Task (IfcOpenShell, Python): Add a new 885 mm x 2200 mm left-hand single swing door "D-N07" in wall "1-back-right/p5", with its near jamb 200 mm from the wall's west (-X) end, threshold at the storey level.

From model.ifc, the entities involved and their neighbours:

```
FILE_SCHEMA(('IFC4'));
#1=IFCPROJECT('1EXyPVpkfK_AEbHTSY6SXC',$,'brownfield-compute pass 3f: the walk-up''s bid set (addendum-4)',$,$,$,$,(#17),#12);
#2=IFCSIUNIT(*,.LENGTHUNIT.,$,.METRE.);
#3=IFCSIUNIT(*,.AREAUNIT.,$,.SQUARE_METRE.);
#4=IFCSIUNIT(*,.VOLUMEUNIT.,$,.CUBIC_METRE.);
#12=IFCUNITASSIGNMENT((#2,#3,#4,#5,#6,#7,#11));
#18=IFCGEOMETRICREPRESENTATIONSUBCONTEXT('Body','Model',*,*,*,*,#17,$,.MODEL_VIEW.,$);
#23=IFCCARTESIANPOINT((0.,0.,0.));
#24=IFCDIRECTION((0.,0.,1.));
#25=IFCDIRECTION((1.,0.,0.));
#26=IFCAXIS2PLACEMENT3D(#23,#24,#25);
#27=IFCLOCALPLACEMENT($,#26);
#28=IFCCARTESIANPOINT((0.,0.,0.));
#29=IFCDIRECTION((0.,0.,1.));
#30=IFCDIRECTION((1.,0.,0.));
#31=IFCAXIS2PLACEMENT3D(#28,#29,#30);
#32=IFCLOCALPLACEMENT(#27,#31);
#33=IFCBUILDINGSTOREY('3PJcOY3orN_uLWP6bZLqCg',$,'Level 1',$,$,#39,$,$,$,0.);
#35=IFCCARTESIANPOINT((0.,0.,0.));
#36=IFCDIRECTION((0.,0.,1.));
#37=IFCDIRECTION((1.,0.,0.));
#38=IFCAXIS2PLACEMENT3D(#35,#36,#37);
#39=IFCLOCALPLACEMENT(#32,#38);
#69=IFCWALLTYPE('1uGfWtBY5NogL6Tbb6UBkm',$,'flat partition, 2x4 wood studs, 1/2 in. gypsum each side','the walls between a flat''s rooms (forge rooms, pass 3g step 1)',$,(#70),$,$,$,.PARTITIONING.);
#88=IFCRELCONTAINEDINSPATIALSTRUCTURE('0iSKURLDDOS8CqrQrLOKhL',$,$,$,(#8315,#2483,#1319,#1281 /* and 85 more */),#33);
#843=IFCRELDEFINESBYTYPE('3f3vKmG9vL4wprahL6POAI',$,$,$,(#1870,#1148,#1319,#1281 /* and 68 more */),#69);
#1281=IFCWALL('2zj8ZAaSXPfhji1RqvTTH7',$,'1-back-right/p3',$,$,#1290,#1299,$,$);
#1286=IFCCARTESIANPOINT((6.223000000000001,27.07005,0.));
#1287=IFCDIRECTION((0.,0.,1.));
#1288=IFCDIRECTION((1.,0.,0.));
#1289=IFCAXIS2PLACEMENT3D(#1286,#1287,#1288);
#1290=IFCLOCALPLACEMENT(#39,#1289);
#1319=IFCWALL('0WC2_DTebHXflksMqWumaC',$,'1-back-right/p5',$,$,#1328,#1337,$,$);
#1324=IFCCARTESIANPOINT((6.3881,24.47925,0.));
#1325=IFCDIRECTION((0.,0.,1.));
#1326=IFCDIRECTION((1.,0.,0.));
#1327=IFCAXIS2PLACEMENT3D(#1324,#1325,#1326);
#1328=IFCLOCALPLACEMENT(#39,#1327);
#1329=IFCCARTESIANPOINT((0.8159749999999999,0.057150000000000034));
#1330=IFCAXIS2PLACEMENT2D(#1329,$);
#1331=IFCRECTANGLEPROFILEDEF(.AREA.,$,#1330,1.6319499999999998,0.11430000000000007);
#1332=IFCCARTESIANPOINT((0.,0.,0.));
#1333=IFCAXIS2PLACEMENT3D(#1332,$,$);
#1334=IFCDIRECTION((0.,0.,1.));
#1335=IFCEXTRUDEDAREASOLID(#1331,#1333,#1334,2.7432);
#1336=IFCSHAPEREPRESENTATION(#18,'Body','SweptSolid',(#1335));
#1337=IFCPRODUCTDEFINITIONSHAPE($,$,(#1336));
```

```python
import numpy as np
import ifcopenshell
import ifcopenshell.api.feature
import ifcopenshell.api.geometry
import ifcopenshell.api.root
import ifcopenshell.api.spatial
import ifcopenshell.geom
import ifcopenshell.util.element
import ifcopenshell.util.placement
import ifcopenshell.util.representation
import ifcopenshell.util.shape
import ifcopenshell.util.unit

model = ifcopenshell.open("model.ifc")
unit_scale = ifcopenshell.util.unit.calculate_unit_scale(model)
settings = ifcopenshell.geom.settings()


def volume(element):
    """Net volume in cubic metres, openings subtracted."""
    shape = ifcopenshell.geom.create_shape(settings, element)
    return ifcopenshell.util.shape.get_volume(shape.geometry)


wall = model.by_guid("0WC2_DTebHXflksMqWumaC")
storey = ifcopenshell.util.element.get_container(wall, ifc_class="IfcBuildingStorey")
context = ifcopenshell.util.representation.get_context(model, "Model", "Body", "MODEL_VIEW")
before = volume(wall)

width, height, from_end, sill = 0.885, 2.2, 0.2, 0.0  # metres

# The wall runs along its own X axis, and the end named is its -X end.
wall_shape = ifcopenshell.geom.create_shape(settings, wall)
x, y, z = ifcopenshell.util.shape.get_vertices(wall_shape.geometry).T
start = x.min() + from_end
face, thickness = float(y.min()), float(y.max() - y.min())
wall_matrix = ifcopenshell.util.placement.get_local_placement(wall.ObjectPlacement)
level = ifcopenshell.util.placement.get_local_placement(storey.ObjectPlacement)[2, 3]


def in_wall(x, y):
    """Placement at x, y metres in the wall's axes, at sill height."""
    matrix = wall_matrix.copy()
    matrix[:, 3] = wall_matrix @ np.array([x / unit_scale, y / unit_scale, 0.0, 1.0])
    matrix[2, 3] = level + sill / unit_scale
    return matrix


# Opening: a box that overshoots both wall faces by 50 mm.
opening = ifcopenshell.api.root.create_entity(model, ifc_class="IfcOpeningElement", predefined_type="OPENING")
box = ifcopenshell.api.geometry.add_wall_representation(
    model, context=context, length=width, height=height, thickness=thickness + 0.1
)
ifcopenshell.api.geometry.assign_representation(model, product=opening, representation=box)
ifcopenshell.api.geometry.edit_object_placement(model, product=opening, matrix=in_wall(start, face - 0.05), is_si=False)
ifcopenshell.api.feature.add_feature(model, feature=opening, element=wall)

door = ifcopenshell.api.root.create_entity(model, ifc_class="IfcDoor", name="D-N07", predefined_type="DOOR")
door.OverallWidth, door.OverallHeight = width / unit_scale, height / unit_scale
door.OperationType = "SINGLE_SWING_LEFT"
body = ifcopenshell.api.geometry.add_door_representation(
    model,
    context=context,
    overall_width=door.OverallWidth,
    overall_height=door.OverallHeight,
    operation_type="SINGLE_SWING_LEFT",
    lining_properties={"LiningDepth": thickness / unit_scale, "ThresholdDepth": thickness / unit_scale},
)
ifcopenshell.api.geometry.assign_representation(model, product=door, representation=body)
ifcopenshell.api.spatial.assign_container(model, products=[door], relating_structure=storey)
ifcopenshell.api.feature.add_filling(model, opening=opening, element=door)

# The lining spans the wall, so the door starts at the wall face.
ifcopenshell.api.geometry.edit_object_placement(model, product=door, matrix=in_wall(start, face), is_si=False)

after = volume(wall)

print(f"wall volume {before:.3f} -> {after:.3f} m3")

model.write("model_updated.ifc")
```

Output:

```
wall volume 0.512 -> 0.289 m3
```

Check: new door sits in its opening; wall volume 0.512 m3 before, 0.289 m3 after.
